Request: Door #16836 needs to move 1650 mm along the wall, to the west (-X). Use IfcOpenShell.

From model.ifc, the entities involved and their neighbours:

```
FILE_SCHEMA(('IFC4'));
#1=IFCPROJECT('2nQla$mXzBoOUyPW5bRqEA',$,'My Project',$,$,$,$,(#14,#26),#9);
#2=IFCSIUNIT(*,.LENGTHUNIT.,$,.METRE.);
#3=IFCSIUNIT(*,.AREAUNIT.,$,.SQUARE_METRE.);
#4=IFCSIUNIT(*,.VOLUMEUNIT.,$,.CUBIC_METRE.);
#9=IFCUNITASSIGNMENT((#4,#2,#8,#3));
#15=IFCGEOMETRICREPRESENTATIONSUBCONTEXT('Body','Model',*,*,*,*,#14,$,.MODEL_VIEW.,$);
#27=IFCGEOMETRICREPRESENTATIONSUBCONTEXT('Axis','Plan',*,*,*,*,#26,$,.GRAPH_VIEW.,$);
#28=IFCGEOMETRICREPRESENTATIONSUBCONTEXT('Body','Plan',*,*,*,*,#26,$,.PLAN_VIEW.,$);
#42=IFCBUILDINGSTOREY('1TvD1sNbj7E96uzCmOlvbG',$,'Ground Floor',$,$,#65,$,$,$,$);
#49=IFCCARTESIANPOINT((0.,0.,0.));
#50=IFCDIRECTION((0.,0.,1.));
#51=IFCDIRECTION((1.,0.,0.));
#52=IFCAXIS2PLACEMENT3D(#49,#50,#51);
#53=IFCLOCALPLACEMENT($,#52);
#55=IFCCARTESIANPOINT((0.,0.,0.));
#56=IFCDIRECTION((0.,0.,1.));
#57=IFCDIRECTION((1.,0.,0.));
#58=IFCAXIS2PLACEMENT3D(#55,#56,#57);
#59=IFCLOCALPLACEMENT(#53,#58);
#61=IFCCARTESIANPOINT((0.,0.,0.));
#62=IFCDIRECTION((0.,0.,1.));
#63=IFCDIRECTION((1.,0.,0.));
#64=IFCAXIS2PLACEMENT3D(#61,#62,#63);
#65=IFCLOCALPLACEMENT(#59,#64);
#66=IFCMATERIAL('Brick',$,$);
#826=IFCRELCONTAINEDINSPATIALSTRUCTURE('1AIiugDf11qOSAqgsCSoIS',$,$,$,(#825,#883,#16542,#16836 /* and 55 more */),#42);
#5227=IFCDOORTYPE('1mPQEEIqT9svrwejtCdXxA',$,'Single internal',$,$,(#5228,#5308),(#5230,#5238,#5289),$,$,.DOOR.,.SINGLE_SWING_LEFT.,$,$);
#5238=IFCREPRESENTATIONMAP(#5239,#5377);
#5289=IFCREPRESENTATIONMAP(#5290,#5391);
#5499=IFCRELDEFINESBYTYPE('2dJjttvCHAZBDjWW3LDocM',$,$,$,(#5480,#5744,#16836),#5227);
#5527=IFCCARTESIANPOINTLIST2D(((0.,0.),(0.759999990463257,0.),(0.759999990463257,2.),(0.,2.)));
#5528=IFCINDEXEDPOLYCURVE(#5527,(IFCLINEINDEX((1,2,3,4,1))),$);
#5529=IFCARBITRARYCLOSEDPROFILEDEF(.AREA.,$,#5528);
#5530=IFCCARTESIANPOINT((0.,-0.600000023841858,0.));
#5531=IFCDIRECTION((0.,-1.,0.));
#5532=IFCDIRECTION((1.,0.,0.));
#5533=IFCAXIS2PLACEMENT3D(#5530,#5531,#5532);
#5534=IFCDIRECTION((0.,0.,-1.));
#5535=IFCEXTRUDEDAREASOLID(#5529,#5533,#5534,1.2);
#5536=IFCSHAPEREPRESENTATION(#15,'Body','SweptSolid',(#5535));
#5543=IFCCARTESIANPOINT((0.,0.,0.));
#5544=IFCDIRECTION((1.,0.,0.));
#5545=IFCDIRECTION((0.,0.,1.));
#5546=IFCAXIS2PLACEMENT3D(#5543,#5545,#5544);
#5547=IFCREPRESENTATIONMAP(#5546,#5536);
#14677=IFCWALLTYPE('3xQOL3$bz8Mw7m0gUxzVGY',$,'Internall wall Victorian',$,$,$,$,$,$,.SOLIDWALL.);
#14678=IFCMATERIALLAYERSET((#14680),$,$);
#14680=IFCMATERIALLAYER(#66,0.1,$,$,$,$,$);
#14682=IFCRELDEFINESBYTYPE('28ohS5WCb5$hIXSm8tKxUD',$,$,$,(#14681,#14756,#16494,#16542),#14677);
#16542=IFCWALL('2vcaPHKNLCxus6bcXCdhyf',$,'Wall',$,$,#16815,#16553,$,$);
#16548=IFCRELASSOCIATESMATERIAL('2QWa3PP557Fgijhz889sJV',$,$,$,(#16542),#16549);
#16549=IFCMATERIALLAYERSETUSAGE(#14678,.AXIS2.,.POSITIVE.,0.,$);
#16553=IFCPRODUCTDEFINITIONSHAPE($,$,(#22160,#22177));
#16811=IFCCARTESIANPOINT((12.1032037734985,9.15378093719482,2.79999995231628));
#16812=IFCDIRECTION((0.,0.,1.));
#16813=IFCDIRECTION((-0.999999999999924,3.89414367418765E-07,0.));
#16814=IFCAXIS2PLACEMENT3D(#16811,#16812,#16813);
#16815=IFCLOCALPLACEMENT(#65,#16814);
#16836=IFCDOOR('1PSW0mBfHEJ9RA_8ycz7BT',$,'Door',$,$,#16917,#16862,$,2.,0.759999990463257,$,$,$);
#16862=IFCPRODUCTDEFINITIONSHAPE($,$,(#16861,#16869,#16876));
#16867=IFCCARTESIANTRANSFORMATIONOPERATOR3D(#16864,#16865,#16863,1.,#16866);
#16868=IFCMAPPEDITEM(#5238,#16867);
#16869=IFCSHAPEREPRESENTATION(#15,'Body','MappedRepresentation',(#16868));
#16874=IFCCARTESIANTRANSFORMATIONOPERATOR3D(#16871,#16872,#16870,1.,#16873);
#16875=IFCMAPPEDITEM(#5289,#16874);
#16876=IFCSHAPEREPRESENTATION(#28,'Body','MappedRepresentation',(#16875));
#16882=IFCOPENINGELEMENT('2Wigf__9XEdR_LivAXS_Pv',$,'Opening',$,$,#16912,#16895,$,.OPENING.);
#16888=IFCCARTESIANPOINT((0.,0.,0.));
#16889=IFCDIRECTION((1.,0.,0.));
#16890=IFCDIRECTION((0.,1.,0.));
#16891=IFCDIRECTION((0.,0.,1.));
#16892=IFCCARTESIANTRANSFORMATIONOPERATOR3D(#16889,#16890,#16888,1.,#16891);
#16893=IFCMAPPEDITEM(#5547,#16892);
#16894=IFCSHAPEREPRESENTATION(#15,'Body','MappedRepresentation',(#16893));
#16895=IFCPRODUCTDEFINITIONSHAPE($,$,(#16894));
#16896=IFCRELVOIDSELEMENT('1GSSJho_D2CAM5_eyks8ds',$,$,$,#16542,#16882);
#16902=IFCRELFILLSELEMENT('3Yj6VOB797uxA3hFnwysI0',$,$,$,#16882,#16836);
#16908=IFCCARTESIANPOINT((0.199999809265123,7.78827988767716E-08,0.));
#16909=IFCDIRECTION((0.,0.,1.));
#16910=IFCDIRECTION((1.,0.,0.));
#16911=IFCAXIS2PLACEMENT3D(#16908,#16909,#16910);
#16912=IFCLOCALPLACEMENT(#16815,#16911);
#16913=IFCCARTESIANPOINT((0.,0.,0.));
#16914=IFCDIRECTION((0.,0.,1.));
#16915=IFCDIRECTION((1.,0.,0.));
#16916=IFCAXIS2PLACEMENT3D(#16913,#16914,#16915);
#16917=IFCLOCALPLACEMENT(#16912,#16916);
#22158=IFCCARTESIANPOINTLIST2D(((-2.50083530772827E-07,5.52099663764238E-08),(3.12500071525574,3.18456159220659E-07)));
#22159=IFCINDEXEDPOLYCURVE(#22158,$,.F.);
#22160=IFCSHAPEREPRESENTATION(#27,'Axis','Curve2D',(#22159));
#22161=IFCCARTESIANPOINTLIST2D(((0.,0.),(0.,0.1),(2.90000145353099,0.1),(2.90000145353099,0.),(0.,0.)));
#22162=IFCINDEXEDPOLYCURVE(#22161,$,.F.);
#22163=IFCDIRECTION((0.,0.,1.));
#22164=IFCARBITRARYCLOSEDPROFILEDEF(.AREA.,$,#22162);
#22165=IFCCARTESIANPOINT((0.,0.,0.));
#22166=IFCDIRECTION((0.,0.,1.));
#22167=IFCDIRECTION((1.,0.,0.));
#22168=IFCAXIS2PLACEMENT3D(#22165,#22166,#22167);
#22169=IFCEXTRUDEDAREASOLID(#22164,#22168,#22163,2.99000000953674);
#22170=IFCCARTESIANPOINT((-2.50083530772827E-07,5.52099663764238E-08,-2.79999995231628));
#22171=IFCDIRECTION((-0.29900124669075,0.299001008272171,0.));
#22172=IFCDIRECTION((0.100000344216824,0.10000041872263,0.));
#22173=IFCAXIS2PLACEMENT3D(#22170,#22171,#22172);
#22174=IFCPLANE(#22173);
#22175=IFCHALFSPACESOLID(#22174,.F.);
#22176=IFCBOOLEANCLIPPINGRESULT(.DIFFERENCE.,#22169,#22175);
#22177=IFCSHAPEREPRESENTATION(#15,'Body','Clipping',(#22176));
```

```python
import ifcopenshell
import ifcopenshell.api.geometry
import ifcopenshell.util.placement

model = ifcopenshell.open("model.ifc")

door = model.by_guid("1PSW0mBfHEJ9RA_8ycz7BT")
opening = door.FillsVoids[0].RelatingOpeningElement
wall = opening.VoidsElements[0].RelatingBuildingElement

wall_matrix = ifcopenshell.util.placement.get_local_placement(wall.ObjectPlacement)
shift = wall_matrix[:3, 0] * 1.65
before = ifcopenshell.util.placement.get_local_placement(door.ObjectPlacement)[:3, 3].copy()

# The door is placed relative to its opening, so it follows when the opening moves.
matrix = ifcopenshell.util.placement.get_local_placement(opening.ObjectPlacement)
matrix[:3, 3] += shift
ifcopenshell.api.geometry.edit_object_placement(
    model, product=opening, matrix=matrix, is_si=False, should_transform_children=True
)

after = ifcopenshell.util.placement.get_local_placement(door.ObjectPlacement)[:3, 3]
print("door moved by", (after - before).round(3) + 0.0)

model.write("model_rev.ifc")
```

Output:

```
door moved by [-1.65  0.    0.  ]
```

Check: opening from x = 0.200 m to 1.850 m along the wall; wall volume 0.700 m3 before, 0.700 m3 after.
